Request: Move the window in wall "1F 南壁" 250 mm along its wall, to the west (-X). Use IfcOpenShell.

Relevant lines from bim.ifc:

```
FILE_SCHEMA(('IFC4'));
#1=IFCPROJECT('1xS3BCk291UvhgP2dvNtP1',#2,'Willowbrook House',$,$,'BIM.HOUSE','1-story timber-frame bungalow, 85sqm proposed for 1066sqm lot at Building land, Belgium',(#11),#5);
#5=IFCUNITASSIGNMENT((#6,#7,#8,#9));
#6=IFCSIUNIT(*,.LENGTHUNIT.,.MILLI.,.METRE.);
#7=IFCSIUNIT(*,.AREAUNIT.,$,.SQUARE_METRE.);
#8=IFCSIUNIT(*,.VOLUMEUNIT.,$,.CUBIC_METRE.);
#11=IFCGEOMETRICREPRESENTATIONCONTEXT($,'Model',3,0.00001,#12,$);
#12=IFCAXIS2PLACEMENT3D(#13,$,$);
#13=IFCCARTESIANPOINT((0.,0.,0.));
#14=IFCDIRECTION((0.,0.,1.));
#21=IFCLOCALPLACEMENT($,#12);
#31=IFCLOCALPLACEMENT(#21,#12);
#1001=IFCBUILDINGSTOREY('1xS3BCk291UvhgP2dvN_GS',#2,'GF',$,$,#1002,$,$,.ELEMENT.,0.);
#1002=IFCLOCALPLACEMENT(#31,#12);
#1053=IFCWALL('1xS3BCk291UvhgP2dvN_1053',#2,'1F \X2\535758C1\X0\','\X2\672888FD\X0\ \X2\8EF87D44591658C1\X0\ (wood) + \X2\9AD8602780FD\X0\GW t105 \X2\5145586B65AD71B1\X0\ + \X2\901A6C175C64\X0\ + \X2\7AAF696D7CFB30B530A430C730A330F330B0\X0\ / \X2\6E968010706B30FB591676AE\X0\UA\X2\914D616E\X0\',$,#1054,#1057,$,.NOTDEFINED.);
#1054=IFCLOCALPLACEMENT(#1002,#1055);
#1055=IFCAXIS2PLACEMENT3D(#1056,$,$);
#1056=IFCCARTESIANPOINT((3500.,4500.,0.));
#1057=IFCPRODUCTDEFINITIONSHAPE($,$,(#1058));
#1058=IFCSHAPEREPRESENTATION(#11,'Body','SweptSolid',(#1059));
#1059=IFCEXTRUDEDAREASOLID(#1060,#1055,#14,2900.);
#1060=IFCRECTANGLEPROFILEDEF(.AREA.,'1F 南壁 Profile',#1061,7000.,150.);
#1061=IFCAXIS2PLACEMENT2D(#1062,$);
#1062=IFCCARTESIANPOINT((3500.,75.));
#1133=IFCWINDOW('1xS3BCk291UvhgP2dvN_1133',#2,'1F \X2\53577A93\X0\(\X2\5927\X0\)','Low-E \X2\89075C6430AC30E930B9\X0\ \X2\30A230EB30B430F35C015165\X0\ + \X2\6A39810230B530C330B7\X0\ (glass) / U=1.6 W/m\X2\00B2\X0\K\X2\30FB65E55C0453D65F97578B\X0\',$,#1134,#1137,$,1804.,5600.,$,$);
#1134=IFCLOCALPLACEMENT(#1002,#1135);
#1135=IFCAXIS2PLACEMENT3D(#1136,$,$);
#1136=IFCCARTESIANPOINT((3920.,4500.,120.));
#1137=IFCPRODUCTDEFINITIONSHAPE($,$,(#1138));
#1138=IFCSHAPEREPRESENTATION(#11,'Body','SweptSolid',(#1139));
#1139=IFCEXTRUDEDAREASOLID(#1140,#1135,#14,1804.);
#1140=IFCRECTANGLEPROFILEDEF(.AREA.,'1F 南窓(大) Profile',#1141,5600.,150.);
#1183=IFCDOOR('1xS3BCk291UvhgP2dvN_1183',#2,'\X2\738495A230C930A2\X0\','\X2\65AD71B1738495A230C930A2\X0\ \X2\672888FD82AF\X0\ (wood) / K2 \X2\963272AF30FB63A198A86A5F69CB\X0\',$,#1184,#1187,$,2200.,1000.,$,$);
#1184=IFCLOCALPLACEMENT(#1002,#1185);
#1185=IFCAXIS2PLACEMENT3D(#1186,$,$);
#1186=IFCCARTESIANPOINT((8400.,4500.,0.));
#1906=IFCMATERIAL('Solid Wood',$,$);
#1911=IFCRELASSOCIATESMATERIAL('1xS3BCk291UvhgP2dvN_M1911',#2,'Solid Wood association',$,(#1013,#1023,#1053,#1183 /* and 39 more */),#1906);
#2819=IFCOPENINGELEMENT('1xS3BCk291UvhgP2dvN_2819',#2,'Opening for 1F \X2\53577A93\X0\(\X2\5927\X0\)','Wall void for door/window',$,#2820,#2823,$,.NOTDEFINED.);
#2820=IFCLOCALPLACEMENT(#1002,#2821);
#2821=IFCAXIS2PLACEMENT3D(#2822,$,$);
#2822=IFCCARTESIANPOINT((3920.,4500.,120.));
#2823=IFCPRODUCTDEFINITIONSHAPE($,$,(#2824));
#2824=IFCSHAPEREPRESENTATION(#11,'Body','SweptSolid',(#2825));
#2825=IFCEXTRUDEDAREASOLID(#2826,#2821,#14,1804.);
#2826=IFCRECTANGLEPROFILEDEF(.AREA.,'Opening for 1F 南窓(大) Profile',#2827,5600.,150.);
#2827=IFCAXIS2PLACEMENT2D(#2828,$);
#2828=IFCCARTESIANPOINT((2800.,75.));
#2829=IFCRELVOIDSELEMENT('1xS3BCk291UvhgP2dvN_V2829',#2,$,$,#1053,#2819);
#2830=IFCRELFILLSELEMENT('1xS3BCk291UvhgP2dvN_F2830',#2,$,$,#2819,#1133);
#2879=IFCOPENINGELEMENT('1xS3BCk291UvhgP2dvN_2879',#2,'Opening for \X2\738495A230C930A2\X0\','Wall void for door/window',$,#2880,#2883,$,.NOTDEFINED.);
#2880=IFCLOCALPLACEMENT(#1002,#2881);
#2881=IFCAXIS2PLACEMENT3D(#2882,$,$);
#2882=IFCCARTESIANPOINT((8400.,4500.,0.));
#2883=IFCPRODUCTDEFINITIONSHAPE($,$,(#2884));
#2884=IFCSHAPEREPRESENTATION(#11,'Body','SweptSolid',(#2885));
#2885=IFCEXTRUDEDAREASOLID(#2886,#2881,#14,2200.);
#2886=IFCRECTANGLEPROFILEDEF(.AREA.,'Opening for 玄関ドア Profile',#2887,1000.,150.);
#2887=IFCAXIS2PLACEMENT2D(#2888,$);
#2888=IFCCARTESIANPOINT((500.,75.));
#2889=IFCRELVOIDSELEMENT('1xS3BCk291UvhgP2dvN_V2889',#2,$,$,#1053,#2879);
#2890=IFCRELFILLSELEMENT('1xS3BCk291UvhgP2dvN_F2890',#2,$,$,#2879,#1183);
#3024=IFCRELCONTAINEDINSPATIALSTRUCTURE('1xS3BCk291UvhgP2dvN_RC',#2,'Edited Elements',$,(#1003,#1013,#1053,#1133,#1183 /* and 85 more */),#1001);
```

```python
import ifcopenshell
import ifcopenshell.api.geometry
import ifcopenshell.util.placement
import ifcopenshell.util.unit

model = ifcopenshell.open("bim.ifc")
unit_scale = ifcopenshell.util.unit.calculate_unit_scale(model)

window = model.by_guid("1xS3BCk291UvhgP2dvN_1133")
opening = window.FillsVoids[0].RelatingOpeningElement
wall = opening.VoidsElements[0].RelatingBuildingElement

wall_matrix = ifcopenshell.util.placement.get_local_placement(wall.ObjectPlacement)
shift = wall_matrix[:3, 0] * -0.25 / unit_scale
before = ifcopenshell.util.placement.get_local_placement(window.ObjectPlacement)[:3, 3].copy()

# The window is not placed relative to its opening, so move both.
for product in (opening, window):
    matrix = ifcopenshell.util.placement.get_local_placement(product.ObjectPlacement)
    matrix[:3, 3] += shift
    ifcopenshell.api.geometry.edit_object_placement(model, product=product, matrix=matrix, is_si=False)

after = ifcopenshell.util.placement.get_local_placement(window.ObjectPlacement)[:3, 3]
print("window moved by", (after - before).round(3) + 0.0)

model.write("bim_rev.ifc")
```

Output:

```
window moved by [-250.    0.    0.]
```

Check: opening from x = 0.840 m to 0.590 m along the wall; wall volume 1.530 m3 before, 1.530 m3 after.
